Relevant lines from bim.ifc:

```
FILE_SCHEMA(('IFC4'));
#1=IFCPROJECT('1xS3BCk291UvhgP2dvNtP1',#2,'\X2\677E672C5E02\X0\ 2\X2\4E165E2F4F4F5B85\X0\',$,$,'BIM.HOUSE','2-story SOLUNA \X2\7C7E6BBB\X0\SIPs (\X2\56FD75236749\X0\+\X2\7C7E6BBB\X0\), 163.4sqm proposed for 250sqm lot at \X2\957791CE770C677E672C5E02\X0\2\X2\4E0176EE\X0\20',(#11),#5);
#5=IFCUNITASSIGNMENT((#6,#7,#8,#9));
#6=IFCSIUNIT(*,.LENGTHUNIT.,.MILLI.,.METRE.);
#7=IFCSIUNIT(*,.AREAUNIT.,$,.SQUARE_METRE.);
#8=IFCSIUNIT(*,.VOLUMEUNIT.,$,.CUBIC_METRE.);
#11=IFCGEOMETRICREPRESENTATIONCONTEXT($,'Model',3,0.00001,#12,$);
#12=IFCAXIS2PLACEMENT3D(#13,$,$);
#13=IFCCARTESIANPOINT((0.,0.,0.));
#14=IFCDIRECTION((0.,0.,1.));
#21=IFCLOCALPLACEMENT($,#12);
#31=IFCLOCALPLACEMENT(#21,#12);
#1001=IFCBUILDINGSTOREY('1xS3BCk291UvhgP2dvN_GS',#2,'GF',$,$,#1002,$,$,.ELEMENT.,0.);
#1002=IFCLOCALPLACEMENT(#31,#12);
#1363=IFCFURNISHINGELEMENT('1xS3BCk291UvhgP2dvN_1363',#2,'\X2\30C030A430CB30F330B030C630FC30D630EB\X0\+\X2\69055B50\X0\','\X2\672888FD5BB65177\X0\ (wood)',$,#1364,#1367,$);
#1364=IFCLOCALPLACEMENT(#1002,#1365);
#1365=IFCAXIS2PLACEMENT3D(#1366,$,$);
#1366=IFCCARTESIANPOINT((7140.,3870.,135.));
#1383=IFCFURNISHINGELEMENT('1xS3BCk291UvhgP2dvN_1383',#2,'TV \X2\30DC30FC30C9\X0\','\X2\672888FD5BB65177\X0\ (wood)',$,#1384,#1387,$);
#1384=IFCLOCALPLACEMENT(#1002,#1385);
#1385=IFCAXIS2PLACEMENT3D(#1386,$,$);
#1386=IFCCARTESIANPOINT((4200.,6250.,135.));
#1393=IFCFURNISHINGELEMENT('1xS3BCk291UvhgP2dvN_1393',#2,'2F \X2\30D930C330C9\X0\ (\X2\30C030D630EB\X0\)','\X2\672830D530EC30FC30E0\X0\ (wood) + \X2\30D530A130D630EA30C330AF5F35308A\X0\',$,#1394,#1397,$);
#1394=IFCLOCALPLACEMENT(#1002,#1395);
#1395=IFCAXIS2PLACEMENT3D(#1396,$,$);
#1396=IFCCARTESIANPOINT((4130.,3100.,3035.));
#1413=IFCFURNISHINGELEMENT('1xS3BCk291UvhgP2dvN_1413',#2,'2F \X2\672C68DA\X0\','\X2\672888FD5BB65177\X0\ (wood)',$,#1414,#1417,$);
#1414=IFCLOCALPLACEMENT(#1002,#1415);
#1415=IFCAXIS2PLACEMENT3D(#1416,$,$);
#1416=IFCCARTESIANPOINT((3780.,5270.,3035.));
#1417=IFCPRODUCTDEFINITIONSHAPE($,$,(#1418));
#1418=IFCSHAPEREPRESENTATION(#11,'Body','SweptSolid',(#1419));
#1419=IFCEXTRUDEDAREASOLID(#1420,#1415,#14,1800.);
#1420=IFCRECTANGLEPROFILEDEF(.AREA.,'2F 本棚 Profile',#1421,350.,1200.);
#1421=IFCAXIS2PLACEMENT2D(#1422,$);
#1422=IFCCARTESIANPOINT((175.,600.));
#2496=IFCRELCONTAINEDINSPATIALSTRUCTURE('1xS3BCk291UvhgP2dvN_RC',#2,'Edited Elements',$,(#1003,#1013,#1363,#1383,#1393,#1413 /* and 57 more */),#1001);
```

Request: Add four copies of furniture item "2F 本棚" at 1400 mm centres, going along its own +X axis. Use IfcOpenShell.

```python
import ifcopenshell
import ifcopenshell.api.geometry
import ifcopenshell.api.root
import ifcopenshell.util.element
import ifcopenshell.util.placement
import ifcopenshell.util.unit

model = ifcopenshell.open("bim.ifc")
unit_scale = ifcopenshell.util.unit.calculate_unit_scale(model)


def reuse_history(source, copy):
    """copy_class also copies each property set's owner history, people and application; keep the originals."""
    for rel in copy.IsDefinedBy:
        if rel.is_a("IfcRelDefinesByProperties") and (history := rel.RelatingPropertyDefinition.OwnerHistory):
            rel.RelatingPropertyDefinition.OwnerHistory = source.OwnerHistory
            ifcopenshell.util.element.remove_deep2(model, history)


source = model.by_guid("1xS3BCk291UvhgP2dvN_1413")
base = ifcopenshell.util.placement.get_local_placement(source.ObjectPlacement)
step = base[:3, 0] * 1.4 / unit_scale

for i in range(1, 5):
    copy = ifcopenshell.api.root.copy_class(model, product=source)
    copy.Representation = ifcopenshell.util.element.copy_deep(
        model, source.Representation, exclude=["IfcGeometricRepresentationContext", "IfcRepresentationMap"]
    )
    reuse_history(source, copy)
    matrix = base.copy()
    matrix[:3, 3] += i * step
    print("added at", matrix[:3, 3].round(3) + 0.0)
    ifcopenshell.api.geometry.edit_object_placement(model, product=copy, matrix=matrix, is_si=False)

model.write("bim_rev.ifc")
```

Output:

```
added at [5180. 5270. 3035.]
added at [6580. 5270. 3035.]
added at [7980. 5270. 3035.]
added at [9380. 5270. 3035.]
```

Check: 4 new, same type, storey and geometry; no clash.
